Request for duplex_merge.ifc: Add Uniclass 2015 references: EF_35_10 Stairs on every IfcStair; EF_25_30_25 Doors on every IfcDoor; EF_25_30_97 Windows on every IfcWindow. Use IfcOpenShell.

First a look at what the model holds.

```python
import ifcopenshell

model = ifcopenshell.open("duplex_merge.ifc")
print(model.schema)
print("classifications:", [c.Name for c in model.by_type("IfcClassification")])
for ifc_class in ("IfcDoor", "IfcRoof", "IfcStair", "IfcWall", "IfcWindow"):
    print(ifc_class, len(model.by_type(ifc_class)))
```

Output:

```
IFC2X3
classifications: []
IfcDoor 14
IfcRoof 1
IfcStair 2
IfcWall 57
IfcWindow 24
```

```python
import ifcopenshell
import ifcopenshell.api.classification

model = ifcopenshell.open("duplex_merge.ifc")

# IFC2X3 requires Source and Edition and has no link from the project to the system.
system = model.create_entity("IfcClassification", Source="NBS", Edition="2015", Name="Uniclass 2015")

codes = {
    "IfcStair": ("EF_35_10", "Stairs"),
    "IfcDoor": ("EF_25_30_25", "Doors"),
    "IfcWindow": ("EF_25_30_97", "Windows"),
}
for ifc_class, (code, name) in codes.items():
    products = model.by_type(ifc_class)
    ifcopenshell.api.classification.add_reference(
        model, products=products, classification=system, identification=code, name=name
    )
    print(code, len(products))

model.write("duplex_merge_v2.ifc")
```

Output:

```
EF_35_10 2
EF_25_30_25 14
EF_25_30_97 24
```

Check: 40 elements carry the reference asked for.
